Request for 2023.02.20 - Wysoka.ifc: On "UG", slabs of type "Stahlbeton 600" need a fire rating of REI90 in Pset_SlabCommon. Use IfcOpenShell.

First a look at what the model holds.

```python
import ifcopenshell
import ifcopenshell.util.element

model = ifcopenshell.open("2023.02.20 - Wysoka.ifc")
print(model.schema)
storey = next(s for s in model.by_type("IfcBuildingStorey") if s.Name == "UG")
slabs = [e for e in ifcopenshell.util.element.get_decomposition(storey) if e.is_a("IfcSlab")]
seen = {}
for e in slabs:
    element_type = ifcopenshell.util.element.get_type(e)
    key = (element_type.Name if element_type != e and element_type else None, ifcopenshell.util.element.get_pset(e, "Pset_SlabCommon", "FireRating"))
    seen[key] = seen.get(key, 0) + 1
for (name, value), count in sorted(seen.items(), key=str):
    print(count, "x", name, "|", value)
```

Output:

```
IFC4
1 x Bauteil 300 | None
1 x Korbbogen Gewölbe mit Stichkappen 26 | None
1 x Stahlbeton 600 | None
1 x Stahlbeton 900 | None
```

```python
import ifcopenshell
import ifcopenshell.api.pset
import ifcopenshell.util.element

model = ifcopenshell.open("2023.02.20 - Wysoka.ifc")

storey = next(s for s in model.by_type("IfcBuildingStorey") if s.Name == "UG")
slabs = [e for e in ifcopenshell.util.element.get_decomposition(storey) if e.is_a("IfcSlab")]

count = 0
for e in slabs:
    element_type = ifcopenshell.util.element.get_type(e)
    if element_type in (None, e) or element_type.Name != "Stahlbeton 600":
        continue
    # add_pset returns the element's existing set when there is one.
    pset = ifcopenshell.api.pset.add_pset(model, product=e, name="Pset_SlabCommon")
    ifcopenshell.api.pset.edit_pset(model, pset=pset, properties={"FireRating": "REI90"})
    count += 1

print(count, "slabs updated")

model.write("2023.02.20 - Wysoka_v2.ifc")
```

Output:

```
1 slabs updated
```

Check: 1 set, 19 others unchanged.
